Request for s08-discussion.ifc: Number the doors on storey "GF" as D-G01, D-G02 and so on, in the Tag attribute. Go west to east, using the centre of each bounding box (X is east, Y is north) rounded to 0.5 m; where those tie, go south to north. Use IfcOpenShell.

First a look at what the model holds.

```python
import ifcopenshell
import ifcopenshell.util.element
import ifcopenshell.util.placement

model = ifcopenshell.open("s08-discussion.ifc")
print(model.schema)
storey = next(s for s in model.by_type("IfcBuildingStorey") if s.Name == "GF")
doors = [e for e in ifcopenshell.util.element.get_decomposition(storey) if e.is_a("IfcDoor")]
for e in sorted(doors, key=lambda e: e.id()):
    origin = ifcopenshell.util.placement.get_local_placement(e.ObjectPlacement)[:3, 3]
    print(e.id(), e.Tag, e.Name, origin.round(2) + 0.0, sep=" | ")
```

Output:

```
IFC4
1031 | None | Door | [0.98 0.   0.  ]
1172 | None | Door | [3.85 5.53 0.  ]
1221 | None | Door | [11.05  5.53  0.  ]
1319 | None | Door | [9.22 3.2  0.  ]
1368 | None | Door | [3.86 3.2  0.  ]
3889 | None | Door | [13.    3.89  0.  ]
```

```python
import ifcopenshell
import ifcopenshell.geom
import ifcopenshell.util.element
import ifcopenshell.util.shape

model = ifcopenshell.open("s08-discussion.ifc")
settings = ifcopenshell.geom.settings()
settings.set("use-world-coords", True)


def centre(element):
    shape = ifcopenshell.geom.create_shape(settings, element)
    return ifcopenshell.util.shape.get_bbox_centroid(shape.geometry)


storey = next(s for s in model.by_type("IfcBuildingStorey") if s.Name == "GF")
doors = [e for e in ifcopenshell.util.element.get_decomposition(storey) if e.is_a("IfcDoor")]

# Insertion points can sit at a corner or the storey origin, so sort by the geometry (in metres).
centres = {e: centre(e) for e in doors}
doors.sort(key=lambda e: (round(centres[e][0] / 0.5), centres[e][1]))

for i, e in enumerate(doors, start=1):
    number = f"D-G{i:02d}"
    e.Tag = number
    print(e.id(), number)

model.write("s08-discussion_v2.ifc")
```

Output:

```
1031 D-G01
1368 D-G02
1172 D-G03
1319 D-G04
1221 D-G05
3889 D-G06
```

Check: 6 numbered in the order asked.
